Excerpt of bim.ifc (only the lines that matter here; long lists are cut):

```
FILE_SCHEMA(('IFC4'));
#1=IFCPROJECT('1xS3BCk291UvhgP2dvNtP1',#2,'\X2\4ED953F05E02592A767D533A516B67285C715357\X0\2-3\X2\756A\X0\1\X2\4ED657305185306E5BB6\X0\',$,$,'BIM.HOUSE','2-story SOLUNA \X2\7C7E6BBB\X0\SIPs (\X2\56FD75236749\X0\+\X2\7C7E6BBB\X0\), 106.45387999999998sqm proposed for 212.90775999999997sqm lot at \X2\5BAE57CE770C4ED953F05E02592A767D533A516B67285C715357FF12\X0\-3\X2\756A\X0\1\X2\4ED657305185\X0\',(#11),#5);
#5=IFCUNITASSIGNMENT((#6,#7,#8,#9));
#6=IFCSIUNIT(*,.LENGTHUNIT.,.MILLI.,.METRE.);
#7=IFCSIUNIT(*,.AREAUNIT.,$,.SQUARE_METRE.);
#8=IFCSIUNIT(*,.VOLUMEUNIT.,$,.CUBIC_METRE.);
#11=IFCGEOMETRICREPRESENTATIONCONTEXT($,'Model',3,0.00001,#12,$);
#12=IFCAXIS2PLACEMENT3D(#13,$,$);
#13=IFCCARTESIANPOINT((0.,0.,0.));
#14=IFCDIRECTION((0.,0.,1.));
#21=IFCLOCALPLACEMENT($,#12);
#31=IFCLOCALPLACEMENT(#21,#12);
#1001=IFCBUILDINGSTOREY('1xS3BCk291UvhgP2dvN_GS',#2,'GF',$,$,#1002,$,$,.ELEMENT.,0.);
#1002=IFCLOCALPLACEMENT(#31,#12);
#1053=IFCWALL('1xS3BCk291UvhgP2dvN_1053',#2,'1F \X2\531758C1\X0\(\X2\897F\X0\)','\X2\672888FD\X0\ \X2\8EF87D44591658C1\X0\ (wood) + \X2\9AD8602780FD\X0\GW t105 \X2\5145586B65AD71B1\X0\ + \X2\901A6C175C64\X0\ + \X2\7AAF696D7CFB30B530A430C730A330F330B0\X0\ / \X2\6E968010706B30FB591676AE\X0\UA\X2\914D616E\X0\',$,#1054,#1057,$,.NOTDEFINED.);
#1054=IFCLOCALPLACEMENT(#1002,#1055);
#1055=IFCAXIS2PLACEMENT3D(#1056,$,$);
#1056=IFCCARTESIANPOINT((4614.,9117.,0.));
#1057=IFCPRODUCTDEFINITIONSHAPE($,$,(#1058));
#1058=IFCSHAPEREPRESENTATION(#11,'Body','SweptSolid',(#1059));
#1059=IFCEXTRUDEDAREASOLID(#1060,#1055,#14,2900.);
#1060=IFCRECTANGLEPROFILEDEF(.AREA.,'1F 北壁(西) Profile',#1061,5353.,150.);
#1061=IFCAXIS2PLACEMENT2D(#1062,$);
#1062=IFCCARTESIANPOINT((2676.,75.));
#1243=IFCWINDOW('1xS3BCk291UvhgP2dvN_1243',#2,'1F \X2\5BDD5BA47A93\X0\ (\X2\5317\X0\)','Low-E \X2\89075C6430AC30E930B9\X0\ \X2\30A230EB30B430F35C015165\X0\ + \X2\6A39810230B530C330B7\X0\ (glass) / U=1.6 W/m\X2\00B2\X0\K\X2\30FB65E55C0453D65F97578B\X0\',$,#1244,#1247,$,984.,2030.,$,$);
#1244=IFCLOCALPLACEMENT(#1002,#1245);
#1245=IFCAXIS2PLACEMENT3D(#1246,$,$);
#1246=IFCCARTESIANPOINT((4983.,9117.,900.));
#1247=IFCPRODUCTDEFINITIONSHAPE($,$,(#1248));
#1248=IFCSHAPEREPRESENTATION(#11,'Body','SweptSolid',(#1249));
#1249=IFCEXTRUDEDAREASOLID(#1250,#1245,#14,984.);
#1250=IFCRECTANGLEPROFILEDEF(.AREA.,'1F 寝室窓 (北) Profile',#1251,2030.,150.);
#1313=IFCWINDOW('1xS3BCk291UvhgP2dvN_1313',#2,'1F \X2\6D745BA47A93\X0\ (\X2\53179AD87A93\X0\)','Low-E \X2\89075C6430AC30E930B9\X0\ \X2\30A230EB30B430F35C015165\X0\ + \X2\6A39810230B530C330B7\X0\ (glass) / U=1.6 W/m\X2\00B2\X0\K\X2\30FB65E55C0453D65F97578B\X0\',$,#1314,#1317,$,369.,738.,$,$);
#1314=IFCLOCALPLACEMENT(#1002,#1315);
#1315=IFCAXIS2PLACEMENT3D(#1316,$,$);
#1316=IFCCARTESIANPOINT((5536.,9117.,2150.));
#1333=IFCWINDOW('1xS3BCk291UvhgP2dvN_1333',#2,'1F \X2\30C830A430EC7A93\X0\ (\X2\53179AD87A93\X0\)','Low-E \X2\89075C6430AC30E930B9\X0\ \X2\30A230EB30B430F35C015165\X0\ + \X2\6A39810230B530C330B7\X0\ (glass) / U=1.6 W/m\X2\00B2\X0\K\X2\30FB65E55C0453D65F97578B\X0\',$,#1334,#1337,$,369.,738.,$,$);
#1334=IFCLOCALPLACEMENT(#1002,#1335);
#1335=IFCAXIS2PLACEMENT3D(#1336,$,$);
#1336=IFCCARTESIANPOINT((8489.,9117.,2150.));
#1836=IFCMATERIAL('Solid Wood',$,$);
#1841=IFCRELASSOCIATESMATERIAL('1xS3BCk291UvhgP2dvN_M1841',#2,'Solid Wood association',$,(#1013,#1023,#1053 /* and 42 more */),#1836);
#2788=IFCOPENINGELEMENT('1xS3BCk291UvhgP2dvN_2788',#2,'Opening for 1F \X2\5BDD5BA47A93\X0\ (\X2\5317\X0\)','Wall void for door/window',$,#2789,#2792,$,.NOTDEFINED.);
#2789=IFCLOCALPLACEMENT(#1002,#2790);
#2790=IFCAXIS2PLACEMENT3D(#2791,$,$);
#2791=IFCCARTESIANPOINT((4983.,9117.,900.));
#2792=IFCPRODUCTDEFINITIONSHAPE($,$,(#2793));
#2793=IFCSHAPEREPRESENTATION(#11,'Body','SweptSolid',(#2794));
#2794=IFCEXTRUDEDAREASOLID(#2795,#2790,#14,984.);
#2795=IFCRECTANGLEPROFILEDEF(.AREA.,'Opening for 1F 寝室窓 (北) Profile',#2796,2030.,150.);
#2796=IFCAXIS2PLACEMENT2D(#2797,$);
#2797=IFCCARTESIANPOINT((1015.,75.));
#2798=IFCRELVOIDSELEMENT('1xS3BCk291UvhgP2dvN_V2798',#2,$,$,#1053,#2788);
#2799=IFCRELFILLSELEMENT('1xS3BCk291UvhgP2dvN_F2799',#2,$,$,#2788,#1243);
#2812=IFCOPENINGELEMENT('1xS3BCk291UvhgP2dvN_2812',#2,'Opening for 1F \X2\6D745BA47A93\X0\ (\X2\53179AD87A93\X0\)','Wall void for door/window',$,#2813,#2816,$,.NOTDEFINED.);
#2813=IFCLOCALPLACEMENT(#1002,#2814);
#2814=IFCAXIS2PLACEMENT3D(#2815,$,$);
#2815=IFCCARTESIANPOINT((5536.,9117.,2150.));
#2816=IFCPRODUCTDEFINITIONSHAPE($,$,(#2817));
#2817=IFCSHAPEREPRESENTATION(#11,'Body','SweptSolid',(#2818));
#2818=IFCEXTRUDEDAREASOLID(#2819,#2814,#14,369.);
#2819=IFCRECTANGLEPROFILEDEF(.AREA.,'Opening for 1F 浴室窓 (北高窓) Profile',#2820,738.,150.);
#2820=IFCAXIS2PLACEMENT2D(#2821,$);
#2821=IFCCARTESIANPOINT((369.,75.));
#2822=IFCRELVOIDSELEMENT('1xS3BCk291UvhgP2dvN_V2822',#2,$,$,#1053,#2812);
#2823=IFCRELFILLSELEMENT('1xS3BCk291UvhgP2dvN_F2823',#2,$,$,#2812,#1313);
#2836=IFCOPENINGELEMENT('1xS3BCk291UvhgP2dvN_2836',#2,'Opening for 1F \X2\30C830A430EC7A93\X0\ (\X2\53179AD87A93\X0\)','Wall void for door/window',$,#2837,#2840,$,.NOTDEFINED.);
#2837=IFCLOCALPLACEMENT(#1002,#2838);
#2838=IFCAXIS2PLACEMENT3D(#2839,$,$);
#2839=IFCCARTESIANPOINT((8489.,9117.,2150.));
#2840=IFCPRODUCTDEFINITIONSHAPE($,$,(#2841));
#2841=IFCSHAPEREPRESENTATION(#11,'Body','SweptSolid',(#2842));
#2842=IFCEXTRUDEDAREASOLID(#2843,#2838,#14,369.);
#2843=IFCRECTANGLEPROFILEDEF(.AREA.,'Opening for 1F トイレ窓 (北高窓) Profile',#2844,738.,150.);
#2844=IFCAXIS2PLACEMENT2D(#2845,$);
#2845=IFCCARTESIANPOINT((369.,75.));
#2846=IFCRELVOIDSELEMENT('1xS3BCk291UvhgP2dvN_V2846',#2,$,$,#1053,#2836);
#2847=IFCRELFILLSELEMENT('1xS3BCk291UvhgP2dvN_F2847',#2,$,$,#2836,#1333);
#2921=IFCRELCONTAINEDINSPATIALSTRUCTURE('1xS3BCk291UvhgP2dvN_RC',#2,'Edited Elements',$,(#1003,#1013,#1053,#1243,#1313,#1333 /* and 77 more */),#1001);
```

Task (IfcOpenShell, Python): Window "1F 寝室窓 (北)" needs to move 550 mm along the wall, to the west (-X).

```python
import ifcopenshell
import ifcopenshell.api.geometry
import ifcopenshell.util.placement
import ifcopenshell.util.unit

model = ifcopenshell.open("bim.ifc")
unit_scale = ifcopenshell.util.unit.calculate_unit_scale(model)

window = model.by_guid("1xS3BCk291UvhgP2dvN_1243")
opening = window.FillsVoids[0].RelatingOpeningElement
wall = opening.VoidsElements[0].RelatingBuildingElement

wall_matrix = ifcopenshell.util.placement.get_local_placement(wall.ObjectPlacement)
shift = wall_matrix[:3, 0] * -0.55 / unit_scale
before = ifcopenshell.util.placement.get_local_placement(window.ObjectPlacement)[:3, 3].copy()

# The window is not placed relative to its opening, so move both.
for product in (opening, window):
    matrix = ifcopenshell.util.placement.get_local_placement(product.ObjectPlacement)
    matrix[:3, 3] += shift
    ifcopenshell.api.geometry.edit_object_placement(model, product=product, matrix=matrix, is_si=False)

after = ifcopenshell.util.placement.get_local_placement(window.ObjectPlacement)[:3, 3]
print("window moved by", (after - before).round(3) + 0.0)

model.write("bim_rev.ifc")
```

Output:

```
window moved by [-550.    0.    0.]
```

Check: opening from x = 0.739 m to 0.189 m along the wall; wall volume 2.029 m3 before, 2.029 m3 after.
